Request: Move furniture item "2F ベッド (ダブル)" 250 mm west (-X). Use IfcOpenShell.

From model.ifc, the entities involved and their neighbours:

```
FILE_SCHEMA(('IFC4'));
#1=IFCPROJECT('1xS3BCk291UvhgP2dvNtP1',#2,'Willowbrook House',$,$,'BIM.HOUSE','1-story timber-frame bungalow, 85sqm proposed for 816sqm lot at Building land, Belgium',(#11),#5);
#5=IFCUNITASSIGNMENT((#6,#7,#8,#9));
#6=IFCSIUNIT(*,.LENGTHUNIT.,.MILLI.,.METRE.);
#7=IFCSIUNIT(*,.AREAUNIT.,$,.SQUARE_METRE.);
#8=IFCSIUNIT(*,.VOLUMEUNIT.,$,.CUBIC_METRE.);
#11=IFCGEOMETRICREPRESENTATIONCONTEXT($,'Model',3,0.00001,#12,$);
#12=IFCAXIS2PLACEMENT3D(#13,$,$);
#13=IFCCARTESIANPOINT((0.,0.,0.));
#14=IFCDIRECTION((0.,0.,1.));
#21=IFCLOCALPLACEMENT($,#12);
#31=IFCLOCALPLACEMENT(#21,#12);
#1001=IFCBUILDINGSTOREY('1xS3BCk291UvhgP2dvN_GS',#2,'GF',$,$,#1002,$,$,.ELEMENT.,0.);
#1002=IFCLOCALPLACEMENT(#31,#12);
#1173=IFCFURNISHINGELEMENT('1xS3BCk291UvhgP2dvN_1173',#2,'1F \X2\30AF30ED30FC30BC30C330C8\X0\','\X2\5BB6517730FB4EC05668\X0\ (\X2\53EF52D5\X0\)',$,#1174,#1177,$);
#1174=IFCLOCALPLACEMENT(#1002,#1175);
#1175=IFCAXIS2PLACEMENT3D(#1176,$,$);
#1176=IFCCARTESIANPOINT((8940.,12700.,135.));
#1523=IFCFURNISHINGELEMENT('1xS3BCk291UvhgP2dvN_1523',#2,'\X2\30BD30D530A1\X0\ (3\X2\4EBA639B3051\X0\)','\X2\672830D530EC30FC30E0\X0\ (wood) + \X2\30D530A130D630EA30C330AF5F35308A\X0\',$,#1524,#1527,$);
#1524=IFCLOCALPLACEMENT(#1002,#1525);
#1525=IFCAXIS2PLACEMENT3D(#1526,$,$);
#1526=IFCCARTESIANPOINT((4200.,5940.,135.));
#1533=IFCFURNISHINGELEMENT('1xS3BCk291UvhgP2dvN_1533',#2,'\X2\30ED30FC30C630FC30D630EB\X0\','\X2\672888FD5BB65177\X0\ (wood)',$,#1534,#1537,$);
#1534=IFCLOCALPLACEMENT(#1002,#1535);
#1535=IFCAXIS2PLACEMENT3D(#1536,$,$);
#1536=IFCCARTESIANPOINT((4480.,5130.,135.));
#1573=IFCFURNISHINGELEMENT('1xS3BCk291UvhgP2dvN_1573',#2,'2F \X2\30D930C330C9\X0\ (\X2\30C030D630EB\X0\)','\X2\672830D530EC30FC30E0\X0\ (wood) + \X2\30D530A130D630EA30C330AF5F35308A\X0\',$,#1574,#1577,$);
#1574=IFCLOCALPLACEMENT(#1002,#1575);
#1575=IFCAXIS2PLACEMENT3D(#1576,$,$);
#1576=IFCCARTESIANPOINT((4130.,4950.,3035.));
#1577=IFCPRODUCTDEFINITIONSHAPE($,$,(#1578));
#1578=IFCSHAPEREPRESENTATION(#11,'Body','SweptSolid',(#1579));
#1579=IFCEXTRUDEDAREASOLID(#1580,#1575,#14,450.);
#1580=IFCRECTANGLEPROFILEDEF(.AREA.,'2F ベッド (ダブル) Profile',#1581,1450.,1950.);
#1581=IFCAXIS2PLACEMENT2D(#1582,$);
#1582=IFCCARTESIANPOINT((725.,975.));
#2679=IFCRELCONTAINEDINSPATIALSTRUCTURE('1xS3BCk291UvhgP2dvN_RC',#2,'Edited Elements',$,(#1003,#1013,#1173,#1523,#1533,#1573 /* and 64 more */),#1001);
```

```python
import ifcopenshell
import ifcopenshell.api.geometry
import ifcopenshell.util.placement
import ifcopenshell.util.unit

model = ifcopenshell.open("model.ifc")
unit_scale = ifcopenshell.util.unit.calculate_unit_scale(model)

item = model.by_id(1573)
matrix = ifcopenshell.util.placement.get_local_placement(item.ObjectPlacement)
matrix[0, 3] -= 0.25 / unit_scale
ifcopenshell.api.geometry.edit_object_placement(model, product=item, matrix=matrix, is_si=False)

print(ifcopenshell.util.placement.get_local_placement(item.ObjectPlacement).round(3) + 0.0)

model.write("model_edited.ifc")
```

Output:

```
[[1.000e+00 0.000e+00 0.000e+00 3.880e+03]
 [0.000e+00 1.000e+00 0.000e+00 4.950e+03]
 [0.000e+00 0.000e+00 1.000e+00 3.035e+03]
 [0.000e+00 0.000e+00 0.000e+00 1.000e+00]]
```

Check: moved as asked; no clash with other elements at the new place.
